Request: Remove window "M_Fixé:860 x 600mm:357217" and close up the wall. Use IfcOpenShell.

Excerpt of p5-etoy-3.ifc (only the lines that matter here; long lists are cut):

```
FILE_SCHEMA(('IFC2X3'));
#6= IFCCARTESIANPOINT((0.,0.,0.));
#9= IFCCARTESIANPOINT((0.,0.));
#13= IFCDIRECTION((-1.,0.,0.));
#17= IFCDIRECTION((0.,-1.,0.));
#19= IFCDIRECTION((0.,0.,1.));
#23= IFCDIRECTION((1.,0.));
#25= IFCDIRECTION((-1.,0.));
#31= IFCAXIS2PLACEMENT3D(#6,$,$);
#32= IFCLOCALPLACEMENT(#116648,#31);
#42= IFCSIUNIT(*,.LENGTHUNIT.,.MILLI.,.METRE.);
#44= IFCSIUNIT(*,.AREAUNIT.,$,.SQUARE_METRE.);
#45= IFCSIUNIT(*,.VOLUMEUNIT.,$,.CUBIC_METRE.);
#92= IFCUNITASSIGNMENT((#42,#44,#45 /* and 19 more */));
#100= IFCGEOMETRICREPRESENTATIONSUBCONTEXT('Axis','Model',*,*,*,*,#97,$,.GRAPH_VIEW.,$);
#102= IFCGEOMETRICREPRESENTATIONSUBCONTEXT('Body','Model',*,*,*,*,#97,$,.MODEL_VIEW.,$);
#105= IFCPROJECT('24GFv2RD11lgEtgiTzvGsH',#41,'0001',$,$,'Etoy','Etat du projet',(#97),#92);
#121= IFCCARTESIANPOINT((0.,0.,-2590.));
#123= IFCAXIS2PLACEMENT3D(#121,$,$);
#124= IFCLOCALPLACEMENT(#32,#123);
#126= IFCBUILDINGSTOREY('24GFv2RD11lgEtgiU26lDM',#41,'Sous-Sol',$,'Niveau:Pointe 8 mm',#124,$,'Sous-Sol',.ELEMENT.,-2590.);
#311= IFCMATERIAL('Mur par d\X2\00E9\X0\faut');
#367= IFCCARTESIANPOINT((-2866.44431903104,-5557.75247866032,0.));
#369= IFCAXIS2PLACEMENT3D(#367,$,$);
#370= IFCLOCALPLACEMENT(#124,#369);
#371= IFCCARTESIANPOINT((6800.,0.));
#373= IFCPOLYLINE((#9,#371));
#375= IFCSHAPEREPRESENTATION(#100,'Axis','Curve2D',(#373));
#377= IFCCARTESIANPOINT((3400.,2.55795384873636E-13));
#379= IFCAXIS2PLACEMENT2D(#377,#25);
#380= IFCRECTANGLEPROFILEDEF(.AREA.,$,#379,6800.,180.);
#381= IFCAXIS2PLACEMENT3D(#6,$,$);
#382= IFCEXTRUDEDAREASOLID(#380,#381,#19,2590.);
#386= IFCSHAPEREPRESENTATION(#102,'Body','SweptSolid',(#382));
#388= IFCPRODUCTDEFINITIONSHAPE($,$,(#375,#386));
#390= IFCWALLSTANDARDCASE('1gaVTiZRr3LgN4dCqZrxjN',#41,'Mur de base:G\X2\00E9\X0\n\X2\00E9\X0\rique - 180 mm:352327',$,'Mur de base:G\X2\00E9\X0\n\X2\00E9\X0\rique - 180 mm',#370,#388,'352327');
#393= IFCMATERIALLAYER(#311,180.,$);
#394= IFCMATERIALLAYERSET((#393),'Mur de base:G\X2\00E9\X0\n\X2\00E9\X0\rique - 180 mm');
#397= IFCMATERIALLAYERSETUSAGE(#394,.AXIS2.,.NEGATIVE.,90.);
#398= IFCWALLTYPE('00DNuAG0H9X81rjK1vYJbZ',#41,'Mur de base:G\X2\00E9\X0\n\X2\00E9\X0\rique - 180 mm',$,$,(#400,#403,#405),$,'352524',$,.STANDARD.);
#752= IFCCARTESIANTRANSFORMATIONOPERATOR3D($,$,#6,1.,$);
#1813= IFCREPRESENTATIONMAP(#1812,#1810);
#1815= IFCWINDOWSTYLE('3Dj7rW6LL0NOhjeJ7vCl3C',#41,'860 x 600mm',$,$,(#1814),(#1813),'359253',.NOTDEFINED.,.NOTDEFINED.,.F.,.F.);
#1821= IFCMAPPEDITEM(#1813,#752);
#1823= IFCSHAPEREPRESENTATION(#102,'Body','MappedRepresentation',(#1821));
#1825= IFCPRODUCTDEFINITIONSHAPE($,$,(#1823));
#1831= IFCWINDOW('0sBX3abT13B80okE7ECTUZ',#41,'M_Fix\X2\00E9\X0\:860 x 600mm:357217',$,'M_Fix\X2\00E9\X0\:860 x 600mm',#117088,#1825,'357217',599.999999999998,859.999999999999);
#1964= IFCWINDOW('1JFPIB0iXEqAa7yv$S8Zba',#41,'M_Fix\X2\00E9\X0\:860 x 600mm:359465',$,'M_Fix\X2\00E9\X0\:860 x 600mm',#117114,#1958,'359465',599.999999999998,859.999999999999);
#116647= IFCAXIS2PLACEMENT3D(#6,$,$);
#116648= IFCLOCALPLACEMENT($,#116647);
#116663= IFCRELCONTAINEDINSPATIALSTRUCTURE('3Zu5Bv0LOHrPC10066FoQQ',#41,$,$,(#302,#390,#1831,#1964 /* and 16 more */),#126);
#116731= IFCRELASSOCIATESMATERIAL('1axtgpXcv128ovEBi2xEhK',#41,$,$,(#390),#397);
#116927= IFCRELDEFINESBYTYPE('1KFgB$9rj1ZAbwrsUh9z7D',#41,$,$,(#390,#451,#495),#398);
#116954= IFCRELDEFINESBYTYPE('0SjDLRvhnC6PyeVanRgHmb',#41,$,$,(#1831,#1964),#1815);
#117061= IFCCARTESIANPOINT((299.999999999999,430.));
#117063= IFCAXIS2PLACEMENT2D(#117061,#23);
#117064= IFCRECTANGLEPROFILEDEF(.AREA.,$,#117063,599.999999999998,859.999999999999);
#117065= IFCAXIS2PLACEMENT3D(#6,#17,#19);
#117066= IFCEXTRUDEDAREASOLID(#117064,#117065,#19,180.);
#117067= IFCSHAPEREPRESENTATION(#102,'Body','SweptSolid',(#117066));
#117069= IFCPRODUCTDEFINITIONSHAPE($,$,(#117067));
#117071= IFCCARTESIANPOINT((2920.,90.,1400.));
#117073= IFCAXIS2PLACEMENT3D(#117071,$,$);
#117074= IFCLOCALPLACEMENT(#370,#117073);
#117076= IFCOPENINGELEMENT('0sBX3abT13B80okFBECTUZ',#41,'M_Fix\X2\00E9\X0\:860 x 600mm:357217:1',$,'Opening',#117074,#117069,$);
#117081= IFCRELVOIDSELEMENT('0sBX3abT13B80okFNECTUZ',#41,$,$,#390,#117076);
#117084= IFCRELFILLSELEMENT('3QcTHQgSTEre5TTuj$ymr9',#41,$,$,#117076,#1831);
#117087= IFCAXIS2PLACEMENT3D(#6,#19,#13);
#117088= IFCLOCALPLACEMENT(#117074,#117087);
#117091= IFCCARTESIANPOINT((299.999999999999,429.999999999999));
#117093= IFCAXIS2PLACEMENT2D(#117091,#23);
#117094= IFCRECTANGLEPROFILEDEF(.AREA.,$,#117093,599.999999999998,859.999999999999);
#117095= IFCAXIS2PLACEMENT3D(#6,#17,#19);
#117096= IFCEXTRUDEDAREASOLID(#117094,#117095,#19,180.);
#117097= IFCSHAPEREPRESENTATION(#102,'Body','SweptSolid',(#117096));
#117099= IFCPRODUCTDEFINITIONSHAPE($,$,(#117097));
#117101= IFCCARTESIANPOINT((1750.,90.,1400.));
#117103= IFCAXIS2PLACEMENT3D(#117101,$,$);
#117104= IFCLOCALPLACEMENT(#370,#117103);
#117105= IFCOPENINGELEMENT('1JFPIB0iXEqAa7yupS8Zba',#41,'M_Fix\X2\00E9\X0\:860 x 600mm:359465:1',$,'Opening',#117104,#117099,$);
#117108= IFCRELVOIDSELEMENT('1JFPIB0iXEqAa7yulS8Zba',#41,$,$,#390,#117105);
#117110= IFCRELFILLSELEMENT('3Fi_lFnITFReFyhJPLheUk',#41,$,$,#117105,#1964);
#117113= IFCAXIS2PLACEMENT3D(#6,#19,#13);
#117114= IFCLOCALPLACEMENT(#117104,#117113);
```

```python
import ifcopenshell
import ifcopenshell.api.feature
import ifcopenshell.api.root
import ifcopenshell.geom
import ifcopenshell.util.shape

model = ifcopenshell.open("p5-etoy-3.ifc")
settings = ifcopenshell.geom.settings()


def volume(element):
    """Net volume in cubic metres, openings subtracted."""
    shape = ifcopenshell.geom.create_shape(settings, element)
    return ifcopenshell.util.shape.get_volume(shape.geometry)


window = model.by_guid("0sBX3abT13B80okE7ECTUZ")
opening = window.FillsVoids[0].RelatingOpeningElement
wall = opening.VoidsElements[0].RelatingBuildingElement
before = volume(wall)

ifcopenshell.api.root.remove_product(model, product=window)
ifcopenshell.api.feature.remove_feature(model, feature=opening)

after = volume(wall)

print(f"wall volume {before:.3f} -> {after:.3f} m3")

model.write("p5-etoy-3_edited.ifc")
```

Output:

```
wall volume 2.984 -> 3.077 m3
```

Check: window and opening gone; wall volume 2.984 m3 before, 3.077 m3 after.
